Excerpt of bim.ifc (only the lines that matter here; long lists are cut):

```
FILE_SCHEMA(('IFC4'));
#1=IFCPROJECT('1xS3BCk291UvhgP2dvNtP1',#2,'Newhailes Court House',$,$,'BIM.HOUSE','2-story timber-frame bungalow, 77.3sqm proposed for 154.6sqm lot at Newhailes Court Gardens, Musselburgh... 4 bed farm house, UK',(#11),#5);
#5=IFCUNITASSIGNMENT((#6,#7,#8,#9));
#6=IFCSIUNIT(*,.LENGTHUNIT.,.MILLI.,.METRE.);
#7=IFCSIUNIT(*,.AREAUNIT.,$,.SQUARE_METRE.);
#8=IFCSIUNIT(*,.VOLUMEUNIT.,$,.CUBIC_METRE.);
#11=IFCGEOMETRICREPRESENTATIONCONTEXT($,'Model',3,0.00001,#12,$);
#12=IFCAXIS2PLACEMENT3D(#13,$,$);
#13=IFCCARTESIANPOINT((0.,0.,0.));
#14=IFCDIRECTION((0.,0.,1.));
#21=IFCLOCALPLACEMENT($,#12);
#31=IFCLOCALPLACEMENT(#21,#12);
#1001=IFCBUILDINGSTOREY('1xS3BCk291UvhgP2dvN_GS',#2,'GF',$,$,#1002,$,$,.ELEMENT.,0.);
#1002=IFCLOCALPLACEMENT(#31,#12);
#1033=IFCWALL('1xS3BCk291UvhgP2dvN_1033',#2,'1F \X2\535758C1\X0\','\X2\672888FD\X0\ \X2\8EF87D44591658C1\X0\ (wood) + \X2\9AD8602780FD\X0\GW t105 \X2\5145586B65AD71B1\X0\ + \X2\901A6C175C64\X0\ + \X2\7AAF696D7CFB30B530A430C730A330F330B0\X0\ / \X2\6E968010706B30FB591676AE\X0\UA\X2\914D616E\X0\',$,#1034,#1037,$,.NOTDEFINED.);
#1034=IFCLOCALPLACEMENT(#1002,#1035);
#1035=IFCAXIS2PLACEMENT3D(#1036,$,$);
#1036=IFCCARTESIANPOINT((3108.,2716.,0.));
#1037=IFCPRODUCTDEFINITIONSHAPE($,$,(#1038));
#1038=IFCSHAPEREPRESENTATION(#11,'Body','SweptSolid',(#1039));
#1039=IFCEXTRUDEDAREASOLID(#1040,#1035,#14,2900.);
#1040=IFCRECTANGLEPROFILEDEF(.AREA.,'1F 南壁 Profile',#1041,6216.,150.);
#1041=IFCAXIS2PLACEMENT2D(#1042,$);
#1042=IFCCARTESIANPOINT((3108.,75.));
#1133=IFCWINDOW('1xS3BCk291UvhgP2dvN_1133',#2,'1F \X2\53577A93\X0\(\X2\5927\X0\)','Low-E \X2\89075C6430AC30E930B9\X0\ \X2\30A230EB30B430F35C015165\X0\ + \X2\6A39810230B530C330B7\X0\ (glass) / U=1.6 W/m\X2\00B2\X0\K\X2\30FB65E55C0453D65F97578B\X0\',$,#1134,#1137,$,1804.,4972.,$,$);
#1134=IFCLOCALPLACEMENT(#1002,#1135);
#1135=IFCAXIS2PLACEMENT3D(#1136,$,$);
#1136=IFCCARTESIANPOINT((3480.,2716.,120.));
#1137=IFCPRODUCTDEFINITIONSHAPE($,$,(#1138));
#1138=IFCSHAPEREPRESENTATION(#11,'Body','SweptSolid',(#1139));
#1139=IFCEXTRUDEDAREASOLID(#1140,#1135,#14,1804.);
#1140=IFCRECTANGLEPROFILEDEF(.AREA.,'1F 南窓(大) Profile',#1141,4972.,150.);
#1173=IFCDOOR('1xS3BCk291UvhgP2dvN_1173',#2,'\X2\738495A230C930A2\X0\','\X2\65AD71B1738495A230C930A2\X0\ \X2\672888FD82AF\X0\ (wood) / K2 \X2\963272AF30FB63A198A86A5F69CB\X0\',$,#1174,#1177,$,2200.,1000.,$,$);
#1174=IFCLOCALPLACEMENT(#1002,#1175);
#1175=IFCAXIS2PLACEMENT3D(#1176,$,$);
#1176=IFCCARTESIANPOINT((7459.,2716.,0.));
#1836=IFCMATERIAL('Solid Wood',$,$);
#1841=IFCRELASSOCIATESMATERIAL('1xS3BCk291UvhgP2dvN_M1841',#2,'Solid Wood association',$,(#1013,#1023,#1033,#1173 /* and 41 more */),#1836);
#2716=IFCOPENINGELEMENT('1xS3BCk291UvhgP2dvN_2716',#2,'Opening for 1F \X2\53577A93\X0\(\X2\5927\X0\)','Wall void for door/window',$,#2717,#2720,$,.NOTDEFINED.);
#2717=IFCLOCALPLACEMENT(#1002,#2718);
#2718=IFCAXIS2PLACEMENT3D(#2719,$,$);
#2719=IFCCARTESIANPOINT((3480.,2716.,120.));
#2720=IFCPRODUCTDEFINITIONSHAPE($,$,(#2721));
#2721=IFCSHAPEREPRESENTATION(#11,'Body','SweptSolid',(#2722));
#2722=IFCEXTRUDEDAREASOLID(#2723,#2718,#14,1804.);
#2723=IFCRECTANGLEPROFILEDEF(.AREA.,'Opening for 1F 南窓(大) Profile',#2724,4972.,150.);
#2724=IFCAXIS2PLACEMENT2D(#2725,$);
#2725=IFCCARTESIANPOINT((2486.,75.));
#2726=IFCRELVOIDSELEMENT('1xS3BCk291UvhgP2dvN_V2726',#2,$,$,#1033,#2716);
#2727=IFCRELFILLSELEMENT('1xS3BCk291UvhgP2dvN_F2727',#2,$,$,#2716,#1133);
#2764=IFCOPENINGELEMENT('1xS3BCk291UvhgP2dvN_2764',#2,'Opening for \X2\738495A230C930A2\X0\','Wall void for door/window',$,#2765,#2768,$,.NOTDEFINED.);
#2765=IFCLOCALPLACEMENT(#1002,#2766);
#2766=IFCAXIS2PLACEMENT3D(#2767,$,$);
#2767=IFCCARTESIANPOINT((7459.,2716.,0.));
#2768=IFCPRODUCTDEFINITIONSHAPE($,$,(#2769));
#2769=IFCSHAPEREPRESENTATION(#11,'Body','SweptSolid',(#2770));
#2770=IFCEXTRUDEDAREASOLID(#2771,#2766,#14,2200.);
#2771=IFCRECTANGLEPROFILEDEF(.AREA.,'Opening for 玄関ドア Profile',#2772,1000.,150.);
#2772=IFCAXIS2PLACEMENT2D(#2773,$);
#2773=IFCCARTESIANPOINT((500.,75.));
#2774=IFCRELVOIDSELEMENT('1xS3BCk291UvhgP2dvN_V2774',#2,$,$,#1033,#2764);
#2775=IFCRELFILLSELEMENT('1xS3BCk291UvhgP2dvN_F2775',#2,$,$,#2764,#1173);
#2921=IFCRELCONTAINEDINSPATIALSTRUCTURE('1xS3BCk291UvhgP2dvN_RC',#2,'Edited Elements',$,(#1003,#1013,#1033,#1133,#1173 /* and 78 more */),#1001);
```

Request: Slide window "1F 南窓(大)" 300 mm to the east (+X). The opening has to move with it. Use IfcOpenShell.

```python
import ifcopenshell
import ifcopenshell.api.geometry
import ifcopenshell.util.placement

model = ifcopenshell.open("bim.ifc")

window = model.by_guid("1xS3BCk291UvhgP2dvN_1133")
opening = window.FillsVoids[0].RelatingOpeningElement
wall = opening.VoidsElements[0].RelatingBuildingElement

wall_matrix = ifcopenshell.util.placement.get_local_placement(wall.ObjectPlacement)
shift = wall_matrix[:3, 0] * 300.0
before = ifcopenshell.util.placement.get_local_placement(window.ObjectPlacement)[:3, 3].copy()

# The window is not placed relative to its opening, so move both.
for product in (opening, window):
    matrix = ifcopenshell.util.placement.get_local_placement(product.ObjectPlacement)
    matrix[:3, 3] += shift
    ifcopenshell.api.geometry.edit_object_placement(model, product=product, matrix=matrix, is_si=False)

after = ifcopenshell.util.placement.get_local_placement(window.ObjectPlacement)[:3, 3]
print("window moved by", (after - before).round(3) + 0.0)

model.write("bim_v2.ifc")
```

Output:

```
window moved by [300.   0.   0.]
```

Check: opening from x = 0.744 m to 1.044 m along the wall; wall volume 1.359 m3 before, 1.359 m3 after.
